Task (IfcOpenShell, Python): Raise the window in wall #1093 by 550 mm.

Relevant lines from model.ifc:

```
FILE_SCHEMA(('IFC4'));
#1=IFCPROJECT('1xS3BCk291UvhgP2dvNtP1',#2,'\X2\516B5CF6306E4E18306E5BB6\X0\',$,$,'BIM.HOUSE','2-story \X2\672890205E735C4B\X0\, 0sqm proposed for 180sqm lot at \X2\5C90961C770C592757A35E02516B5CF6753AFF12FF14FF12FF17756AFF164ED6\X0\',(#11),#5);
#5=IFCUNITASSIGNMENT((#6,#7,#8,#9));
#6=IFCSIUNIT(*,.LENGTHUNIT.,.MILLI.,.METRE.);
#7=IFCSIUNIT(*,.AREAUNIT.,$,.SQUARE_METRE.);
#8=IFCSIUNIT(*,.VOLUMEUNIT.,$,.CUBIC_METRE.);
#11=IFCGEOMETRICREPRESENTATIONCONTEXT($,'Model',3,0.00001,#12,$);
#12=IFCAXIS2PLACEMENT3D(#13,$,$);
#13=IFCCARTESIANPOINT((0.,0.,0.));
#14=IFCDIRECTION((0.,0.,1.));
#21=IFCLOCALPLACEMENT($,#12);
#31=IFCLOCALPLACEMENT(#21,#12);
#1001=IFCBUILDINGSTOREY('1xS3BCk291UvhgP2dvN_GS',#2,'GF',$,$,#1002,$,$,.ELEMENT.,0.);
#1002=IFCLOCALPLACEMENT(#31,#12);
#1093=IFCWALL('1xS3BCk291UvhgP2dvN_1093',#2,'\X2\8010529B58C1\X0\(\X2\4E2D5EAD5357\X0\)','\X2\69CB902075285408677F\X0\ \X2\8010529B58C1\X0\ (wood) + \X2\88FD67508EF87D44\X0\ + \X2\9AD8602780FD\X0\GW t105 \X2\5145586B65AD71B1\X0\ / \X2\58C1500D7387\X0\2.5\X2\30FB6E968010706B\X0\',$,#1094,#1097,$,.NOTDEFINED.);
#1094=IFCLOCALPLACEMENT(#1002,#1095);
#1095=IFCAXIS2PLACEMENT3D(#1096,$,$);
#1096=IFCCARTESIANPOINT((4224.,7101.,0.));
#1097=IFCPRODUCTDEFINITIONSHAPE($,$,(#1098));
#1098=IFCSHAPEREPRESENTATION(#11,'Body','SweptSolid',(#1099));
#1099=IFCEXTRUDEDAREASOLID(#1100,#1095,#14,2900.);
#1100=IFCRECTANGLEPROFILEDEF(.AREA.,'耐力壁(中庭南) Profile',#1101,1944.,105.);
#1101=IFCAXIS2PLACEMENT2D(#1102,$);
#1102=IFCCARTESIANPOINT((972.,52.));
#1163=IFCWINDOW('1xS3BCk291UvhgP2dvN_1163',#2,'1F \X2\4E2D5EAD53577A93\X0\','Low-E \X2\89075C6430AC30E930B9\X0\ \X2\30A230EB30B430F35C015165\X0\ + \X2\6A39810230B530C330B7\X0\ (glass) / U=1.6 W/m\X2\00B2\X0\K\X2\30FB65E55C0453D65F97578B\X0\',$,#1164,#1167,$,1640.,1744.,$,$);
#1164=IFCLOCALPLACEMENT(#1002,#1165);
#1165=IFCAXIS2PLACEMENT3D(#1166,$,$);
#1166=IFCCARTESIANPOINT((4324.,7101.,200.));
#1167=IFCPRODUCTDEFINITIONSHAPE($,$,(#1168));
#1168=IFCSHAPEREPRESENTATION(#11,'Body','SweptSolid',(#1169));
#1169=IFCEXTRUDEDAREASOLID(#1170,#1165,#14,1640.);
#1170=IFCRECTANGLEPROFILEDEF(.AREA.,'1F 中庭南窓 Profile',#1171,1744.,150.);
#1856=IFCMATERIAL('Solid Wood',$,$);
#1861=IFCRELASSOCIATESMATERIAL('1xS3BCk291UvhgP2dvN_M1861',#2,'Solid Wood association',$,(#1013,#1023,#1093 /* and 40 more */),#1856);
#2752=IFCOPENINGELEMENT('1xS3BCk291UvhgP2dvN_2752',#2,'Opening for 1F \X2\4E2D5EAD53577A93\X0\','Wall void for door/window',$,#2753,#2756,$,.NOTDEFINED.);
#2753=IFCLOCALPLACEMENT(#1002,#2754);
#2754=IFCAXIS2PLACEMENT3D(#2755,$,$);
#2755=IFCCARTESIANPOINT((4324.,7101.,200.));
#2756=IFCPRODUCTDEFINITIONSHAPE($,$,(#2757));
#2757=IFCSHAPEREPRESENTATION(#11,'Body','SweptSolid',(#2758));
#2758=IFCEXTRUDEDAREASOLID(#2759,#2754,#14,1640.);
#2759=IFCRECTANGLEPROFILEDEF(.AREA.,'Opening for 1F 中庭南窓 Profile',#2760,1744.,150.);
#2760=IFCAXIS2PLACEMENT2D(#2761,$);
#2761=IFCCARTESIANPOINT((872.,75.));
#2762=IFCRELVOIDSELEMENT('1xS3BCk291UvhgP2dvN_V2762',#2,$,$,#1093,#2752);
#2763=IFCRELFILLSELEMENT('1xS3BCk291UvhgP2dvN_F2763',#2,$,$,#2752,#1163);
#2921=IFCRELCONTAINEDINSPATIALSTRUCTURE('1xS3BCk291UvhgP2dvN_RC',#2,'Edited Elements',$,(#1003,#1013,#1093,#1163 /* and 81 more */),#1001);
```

```python
import numpy as np
import ifcopenshell
import ifcopenshell.api.geometry
import ifcopenshell.util.placement
import ifcopenshell.util.unit

model = ifcopenshell.open("model.ifc")
unit_scale = ifcopenshell.util.unit.calculate_unit_scale(model)

window = model.by_id(1163)
opening = window.FillsVoids[0].RelatingOpeningElement
dz = 0.55 / unit_scale

shift = np.array([0.0, 0.0, dz])
# The window is not placed relative to its opening, so move both.
for product in (opening, window):
    matrix = ifcopenshell.util.placement.get_local_placement(product.ObjectPlacement)
    matrix[:3, 3] += shift
    ifcopenshell.api.geometry.edit_object_placement(model, product=product, matrix=matrix, is_si=False)

print(f"moved by {dz * unit_scale:+.3f} m")

model.write("model_rev.ifc")
```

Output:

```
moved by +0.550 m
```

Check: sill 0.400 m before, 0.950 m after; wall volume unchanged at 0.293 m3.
